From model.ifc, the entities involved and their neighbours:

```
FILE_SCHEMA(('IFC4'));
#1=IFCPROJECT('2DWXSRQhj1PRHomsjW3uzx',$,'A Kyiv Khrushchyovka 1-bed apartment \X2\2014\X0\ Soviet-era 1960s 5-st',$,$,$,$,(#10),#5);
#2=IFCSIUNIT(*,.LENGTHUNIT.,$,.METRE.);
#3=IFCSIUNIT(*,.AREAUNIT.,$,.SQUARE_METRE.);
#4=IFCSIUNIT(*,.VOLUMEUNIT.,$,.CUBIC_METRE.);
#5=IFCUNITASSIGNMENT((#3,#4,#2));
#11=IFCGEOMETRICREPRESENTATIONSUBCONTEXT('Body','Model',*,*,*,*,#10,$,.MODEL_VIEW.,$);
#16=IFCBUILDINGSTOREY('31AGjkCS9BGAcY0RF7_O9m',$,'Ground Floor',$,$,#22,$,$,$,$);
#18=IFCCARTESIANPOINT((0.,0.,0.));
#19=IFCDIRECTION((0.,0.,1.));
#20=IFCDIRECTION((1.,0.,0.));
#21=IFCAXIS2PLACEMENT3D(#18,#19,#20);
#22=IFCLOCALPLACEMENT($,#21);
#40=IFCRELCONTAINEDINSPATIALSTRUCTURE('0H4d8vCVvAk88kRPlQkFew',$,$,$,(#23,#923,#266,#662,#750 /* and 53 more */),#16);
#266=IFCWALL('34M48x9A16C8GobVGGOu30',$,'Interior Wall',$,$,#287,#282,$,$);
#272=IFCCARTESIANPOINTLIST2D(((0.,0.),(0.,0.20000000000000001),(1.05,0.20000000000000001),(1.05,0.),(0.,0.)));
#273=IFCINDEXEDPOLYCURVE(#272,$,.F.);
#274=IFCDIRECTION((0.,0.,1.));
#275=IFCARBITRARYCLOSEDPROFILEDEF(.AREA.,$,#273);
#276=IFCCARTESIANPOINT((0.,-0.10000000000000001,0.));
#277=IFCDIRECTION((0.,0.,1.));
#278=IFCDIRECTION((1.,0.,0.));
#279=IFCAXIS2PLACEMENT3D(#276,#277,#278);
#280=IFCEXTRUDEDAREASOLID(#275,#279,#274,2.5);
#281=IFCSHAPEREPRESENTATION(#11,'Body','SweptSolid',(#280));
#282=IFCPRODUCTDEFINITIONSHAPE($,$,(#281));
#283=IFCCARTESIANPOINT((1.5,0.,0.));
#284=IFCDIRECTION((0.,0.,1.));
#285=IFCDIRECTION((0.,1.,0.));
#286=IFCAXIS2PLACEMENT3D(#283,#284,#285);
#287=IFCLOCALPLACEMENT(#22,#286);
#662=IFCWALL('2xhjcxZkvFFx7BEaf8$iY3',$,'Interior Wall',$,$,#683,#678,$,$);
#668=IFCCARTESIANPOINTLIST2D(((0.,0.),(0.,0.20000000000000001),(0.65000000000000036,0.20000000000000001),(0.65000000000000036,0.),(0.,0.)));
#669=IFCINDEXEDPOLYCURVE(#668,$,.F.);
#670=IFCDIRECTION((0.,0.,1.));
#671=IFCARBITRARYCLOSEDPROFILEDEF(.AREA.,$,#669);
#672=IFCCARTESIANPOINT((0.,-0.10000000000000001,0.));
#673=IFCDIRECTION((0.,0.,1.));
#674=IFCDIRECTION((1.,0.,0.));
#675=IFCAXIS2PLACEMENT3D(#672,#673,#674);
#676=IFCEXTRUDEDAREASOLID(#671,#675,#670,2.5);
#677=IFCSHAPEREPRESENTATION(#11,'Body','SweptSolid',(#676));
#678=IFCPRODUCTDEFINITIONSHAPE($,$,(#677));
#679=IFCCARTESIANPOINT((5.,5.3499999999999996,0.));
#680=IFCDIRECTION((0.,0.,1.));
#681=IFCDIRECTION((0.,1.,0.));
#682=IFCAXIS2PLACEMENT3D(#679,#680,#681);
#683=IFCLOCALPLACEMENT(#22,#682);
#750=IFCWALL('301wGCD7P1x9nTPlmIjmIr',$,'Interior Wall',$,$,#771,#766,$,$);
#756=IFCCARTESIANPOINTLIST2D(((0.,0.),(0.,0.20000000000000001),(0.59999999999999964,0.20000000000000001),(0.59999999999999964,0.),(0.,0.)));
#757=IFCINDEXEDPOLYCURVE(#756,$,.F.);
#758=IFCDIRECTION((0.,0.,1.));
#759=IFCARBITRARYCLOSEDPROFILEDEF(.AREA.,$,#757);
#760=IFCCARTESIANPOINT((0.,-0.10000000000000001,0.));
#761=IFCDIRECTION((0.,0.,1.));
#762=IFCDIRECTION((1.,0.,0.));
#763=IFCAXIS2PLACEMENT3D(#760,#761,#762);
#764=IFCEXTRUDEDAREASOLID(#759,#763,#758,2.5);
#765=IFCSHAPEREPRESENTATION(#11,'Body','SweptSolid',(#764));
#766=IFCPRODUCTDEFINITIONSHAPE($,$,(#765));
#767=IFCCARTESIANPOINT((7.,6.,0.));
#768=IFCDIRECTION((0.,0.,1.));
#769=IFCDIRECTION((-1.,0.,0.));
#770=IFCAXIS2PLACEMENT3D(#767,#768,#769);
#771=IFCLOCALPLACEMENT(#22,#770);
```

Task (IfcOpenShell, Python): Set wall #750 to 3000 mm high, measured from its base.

```python
import ifcopenshell
import ifcopenshell.geom
import ifcopenshell.util.representation
import ifcopenshell.util.shape
import ifcopenshell.util.unit

model = ifcopenshell.open("model.ifc")
unit_scale = ifcopenshell.util.unit.calculate_unit_scale(model)
settings = ifcopenshell.geom.settings()


def volume(element):
    """Net volume in cubic metres, openings subtracted."""
    shape = ifcopenshell.geom.create_shape(settings, element)
    return ifcopenshell.util.shape.get_volume(shape.geometry)


wall = model.by_guid("301wGCD7P1x9nTPlmIjmIr")
before = volume(wall)

body = ifcopenshell.util.representation.get_representation(wall, "Model", "Body")
solid = body.Items[0]
old_height = solid.Depth
solid.Depth = 3 / unit_scale
after = volume(wall)

print(f"height {old_height:g} -> {solid.Depth:g}, volume {before:.3f} -> {after:.3f} m3")

model.write("model_rev.ifc")
```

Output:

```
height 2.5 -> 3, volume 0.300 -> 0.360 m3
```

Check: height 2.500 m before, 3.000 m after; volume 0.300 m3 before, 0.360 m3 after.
